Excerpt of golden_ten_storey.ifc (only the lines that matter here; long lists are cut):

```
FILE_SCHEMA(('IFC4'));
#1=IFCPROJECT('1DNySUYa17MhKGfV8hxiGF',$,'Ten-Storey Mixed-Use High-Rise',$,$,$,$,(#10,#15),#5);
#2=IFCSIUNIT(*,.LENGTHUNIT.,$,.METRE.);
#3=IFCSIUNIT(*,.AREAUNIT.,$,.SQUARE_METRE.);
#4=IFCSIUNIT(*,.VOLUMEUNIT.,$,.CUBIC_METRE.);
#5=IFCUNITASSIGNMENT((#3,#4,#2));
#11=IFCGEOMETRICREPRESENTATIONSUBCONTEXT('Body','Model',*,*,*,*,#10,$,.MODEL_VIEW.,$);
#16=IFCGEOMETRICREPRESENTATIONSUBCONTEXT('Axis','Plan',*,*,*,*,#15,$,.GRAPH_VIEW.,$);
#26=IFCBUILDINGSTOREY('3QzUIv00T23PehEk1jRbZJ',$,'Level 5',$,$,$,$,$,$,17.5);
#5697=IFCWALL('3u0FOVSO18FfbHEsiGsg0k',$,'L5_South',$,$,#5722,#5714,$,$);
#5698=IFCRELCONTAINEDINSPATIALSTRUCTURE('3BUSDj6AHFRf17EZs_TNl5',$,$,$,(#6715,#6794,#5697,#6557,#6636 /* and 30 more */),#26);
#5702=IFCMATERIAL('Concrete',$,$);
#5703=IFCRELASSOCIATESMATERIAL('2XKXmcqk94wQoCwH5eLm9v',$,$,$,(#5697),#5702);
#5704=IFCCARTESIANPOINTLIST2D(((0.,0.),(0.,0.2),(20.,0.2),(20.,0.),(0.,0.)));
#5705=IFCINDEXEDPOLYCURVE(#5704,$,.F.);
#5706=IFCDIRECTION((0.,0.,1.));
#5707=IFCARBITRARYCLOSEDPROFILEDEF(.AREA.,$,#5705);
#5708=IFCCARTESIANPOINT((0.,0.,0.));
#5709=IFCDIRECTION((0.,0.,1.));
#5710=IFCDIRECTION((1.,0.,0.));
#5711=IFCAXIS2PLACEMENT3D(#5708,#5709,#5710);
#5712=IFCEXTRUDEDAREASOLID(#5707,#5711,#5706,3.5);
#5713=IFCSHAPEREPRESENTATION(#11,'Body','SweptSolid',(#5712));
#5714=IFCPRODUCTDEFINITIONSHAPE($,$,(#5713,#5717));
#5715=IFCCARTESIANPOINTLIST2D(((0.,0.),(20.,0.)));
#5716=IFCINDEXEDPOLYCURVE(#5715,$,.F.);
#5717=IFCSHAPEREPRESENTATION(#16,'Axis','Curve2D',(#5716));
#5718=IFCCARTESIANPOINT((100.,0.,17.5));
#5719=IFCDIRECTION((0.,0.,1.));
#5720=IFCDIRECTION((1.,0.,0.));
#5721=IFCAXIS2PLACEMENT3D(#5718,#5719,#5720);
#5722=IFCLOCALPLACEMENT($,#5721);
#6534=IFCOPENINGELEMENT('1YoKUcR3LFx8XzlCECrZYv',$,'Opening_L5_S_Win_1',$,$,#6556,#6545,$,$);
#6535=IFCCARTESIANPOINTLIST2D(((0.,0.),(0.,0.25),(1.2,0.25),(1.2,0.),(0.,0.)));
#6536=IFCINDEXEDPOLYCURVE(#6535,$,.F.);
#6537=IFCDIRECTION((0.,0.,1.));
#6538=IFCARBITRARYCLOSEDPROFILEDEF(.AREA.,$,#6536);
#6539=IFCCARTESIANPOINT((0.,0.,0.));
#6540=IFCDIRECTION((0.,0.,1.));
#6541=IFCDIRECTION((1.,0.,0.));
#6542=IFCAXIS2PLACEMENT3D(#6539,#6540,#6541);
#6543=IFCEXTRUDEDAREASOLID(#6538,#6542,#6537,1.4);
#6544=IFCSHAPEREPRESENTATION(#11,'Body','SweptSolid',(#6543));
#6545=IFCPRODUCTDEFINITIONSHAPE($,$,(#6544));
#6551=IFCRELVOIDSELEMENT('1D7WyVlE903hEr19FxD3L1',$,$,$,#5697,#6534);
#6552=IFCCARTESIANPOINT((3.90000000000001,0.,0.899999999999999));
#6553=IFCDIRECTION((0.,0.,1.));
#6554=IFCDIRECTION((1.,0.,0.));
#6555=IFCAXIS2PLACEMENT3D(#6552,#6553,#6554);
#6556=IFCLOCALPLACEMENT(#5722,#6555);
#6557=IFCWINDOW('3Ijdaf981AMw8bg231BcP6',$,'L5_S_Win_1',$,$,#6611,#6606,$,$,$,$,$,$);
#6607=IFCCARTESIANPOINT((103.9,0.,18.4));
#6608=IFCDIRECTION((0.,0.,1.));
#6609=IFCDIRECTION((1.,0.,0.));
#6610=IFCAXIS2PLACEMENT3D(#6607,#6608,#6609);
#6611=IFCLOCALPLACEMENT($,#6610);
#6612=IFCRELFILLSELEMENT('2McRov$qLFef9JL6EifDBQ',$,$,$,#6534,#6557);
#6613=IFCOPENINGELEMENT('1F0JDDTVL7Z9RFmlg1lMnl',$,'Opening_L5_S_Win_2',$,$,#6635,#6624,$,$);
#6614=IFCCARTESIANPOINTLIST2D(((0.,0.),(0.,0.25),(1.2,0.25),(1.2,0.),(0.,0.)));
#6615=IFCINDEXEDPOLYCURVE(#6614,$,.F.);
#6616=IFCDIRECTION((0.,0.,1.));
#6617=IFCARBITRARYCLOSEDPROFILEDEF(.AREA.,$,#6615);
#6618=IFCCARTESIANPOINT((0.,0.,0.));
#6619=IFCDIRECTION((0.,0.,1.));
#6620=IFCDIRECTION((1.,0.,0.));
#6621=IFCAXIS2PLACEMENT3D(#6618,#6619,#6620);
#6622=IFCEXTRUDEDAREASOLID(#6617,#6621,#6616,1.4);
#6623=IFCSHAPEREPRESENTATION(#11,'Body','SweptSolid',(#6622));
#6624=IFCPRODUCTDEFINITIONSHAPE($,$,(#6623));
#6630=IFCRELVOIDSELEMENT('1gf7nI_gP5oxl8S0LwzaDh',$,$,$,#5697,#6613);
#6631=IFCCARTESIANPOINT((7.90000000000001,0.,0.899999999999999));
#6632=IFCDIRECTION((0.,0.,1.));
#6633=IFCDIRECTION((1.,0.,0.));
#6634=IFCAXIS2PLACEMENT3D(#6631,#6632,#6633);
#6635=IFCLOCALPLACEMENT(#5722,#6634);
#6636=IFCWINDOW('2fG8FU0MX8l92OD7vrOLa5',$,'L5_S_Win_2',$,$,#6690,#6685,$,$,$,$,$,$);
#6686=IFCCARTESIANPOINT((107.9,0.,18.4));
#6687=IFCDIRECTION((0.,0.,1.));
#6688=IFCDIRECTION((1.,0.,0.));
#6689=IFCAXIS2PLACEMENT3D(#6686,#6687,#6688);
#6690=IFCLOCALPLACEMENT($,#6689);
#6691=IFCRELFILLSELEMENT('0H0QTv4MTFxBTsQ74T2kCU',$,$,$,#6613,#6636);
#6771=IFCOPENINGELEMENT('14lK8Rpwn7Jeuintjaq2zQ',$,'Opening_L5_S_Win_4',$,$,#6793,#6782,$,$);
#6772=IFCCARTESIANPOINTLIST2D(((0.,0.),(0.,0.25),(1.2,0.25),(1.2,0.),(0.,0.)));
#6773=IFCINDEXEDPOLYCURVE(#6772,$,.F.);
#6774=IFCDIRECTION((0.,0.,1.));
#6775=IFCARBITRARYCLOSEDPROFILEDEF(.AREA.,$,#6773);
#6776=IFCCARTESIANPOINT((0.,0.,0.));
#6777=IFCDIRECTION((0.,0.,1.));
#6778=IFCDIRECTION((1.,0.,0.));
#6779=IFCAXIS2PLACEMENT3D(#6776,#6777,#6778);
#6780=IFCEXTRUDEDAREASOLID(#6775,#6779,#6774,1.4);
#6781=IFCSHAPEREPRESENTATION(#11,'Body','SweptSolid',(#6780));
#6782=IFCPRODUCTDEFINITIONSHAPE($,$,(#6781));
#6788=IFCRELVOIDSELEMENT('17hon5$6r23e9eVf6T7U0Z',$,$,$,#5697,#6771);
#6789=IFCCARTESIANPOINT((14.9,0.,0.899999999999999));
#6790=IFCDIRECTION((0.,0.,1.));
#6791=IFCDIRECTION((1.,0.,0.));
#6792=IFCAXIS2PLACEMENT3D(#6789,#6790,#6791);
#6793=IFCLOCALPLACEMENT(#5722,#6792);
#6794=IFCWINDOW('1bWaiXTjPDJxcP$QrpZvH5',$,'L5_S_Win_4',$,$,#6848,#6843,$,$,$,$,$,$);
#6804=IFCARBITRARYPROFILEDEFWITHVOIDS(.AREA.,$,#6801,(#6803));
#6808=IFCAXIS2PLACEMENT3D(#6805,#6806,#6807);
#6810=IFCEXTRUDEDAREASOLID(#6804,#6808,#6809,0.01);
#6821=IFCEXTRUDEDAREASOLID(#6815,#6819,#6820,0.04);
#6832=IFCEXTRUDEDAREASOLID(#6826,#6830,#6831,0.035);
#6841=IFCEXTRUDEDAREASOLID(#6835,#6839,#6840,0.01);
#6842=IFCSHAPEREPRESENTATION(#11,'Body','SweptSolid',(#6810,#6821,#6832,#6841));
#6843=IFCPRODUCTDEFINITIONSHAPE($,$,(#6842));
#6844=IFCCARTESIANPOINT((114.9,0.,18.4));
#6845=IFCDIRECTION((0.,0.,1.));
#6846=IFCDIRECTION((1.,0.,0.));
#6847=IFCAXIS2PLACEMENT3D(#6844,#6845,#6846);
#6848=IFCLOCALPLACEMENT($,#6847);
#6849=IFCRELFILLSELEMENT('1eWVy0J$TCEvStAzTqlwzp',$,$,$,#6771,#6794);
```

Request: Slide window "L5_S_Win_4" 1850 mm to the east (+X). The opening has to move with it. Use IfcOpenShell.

```python
import ifcopenshell
import ifcopenshell.api.geometry
import ifcopenshell.util.placement
import ifcopenshell.util.unit

model = ifcopenshell.open("golden_ten_storey.ifc")
unit_scale = ifcopenshell.util.unit.calculate_unit_scale(model)

window = model.by_guid("1bWaiXTjPDJxcP$QrpZvH5")
opening = window.FillsVoids[0].RelatingOpeningElement
wall = opening.VoidsElements[0].RelatingBuildingElement

wall_matrix = ifcopenshell.util.placement.get_local_placement(wall.ObjectPlacement)
shift = wall_matrix[:3, 0] * 1.85 / unit_scale
before = ifcopenshell.util.placement.get_local_placement(window.ObjectPlacement)[:3, 3].copy()

# The window is not placed relative to its opening, so move both.
for product in (opening, window):
    matrix = ifcopenshell.util.placement.get_local_placement(product.ObjectPlacement)
    matrix[:3, 3] += shift
    ifcopenshell.api.geometry.edit_object_placement(model, product=product, matrix=matrix, is_si=False)

after = ifcopenshell.util.placement.get_local_placement(window.ObjectPlacement)[:3, 3]
print("window moved by", (after - before).round(3) + 0.0)

model.write("golden_ten_storey_v2.ifc")
```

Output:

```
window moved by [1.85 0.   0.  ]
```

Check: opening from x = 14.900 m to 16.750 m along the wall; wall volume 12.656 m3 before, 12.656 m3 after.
